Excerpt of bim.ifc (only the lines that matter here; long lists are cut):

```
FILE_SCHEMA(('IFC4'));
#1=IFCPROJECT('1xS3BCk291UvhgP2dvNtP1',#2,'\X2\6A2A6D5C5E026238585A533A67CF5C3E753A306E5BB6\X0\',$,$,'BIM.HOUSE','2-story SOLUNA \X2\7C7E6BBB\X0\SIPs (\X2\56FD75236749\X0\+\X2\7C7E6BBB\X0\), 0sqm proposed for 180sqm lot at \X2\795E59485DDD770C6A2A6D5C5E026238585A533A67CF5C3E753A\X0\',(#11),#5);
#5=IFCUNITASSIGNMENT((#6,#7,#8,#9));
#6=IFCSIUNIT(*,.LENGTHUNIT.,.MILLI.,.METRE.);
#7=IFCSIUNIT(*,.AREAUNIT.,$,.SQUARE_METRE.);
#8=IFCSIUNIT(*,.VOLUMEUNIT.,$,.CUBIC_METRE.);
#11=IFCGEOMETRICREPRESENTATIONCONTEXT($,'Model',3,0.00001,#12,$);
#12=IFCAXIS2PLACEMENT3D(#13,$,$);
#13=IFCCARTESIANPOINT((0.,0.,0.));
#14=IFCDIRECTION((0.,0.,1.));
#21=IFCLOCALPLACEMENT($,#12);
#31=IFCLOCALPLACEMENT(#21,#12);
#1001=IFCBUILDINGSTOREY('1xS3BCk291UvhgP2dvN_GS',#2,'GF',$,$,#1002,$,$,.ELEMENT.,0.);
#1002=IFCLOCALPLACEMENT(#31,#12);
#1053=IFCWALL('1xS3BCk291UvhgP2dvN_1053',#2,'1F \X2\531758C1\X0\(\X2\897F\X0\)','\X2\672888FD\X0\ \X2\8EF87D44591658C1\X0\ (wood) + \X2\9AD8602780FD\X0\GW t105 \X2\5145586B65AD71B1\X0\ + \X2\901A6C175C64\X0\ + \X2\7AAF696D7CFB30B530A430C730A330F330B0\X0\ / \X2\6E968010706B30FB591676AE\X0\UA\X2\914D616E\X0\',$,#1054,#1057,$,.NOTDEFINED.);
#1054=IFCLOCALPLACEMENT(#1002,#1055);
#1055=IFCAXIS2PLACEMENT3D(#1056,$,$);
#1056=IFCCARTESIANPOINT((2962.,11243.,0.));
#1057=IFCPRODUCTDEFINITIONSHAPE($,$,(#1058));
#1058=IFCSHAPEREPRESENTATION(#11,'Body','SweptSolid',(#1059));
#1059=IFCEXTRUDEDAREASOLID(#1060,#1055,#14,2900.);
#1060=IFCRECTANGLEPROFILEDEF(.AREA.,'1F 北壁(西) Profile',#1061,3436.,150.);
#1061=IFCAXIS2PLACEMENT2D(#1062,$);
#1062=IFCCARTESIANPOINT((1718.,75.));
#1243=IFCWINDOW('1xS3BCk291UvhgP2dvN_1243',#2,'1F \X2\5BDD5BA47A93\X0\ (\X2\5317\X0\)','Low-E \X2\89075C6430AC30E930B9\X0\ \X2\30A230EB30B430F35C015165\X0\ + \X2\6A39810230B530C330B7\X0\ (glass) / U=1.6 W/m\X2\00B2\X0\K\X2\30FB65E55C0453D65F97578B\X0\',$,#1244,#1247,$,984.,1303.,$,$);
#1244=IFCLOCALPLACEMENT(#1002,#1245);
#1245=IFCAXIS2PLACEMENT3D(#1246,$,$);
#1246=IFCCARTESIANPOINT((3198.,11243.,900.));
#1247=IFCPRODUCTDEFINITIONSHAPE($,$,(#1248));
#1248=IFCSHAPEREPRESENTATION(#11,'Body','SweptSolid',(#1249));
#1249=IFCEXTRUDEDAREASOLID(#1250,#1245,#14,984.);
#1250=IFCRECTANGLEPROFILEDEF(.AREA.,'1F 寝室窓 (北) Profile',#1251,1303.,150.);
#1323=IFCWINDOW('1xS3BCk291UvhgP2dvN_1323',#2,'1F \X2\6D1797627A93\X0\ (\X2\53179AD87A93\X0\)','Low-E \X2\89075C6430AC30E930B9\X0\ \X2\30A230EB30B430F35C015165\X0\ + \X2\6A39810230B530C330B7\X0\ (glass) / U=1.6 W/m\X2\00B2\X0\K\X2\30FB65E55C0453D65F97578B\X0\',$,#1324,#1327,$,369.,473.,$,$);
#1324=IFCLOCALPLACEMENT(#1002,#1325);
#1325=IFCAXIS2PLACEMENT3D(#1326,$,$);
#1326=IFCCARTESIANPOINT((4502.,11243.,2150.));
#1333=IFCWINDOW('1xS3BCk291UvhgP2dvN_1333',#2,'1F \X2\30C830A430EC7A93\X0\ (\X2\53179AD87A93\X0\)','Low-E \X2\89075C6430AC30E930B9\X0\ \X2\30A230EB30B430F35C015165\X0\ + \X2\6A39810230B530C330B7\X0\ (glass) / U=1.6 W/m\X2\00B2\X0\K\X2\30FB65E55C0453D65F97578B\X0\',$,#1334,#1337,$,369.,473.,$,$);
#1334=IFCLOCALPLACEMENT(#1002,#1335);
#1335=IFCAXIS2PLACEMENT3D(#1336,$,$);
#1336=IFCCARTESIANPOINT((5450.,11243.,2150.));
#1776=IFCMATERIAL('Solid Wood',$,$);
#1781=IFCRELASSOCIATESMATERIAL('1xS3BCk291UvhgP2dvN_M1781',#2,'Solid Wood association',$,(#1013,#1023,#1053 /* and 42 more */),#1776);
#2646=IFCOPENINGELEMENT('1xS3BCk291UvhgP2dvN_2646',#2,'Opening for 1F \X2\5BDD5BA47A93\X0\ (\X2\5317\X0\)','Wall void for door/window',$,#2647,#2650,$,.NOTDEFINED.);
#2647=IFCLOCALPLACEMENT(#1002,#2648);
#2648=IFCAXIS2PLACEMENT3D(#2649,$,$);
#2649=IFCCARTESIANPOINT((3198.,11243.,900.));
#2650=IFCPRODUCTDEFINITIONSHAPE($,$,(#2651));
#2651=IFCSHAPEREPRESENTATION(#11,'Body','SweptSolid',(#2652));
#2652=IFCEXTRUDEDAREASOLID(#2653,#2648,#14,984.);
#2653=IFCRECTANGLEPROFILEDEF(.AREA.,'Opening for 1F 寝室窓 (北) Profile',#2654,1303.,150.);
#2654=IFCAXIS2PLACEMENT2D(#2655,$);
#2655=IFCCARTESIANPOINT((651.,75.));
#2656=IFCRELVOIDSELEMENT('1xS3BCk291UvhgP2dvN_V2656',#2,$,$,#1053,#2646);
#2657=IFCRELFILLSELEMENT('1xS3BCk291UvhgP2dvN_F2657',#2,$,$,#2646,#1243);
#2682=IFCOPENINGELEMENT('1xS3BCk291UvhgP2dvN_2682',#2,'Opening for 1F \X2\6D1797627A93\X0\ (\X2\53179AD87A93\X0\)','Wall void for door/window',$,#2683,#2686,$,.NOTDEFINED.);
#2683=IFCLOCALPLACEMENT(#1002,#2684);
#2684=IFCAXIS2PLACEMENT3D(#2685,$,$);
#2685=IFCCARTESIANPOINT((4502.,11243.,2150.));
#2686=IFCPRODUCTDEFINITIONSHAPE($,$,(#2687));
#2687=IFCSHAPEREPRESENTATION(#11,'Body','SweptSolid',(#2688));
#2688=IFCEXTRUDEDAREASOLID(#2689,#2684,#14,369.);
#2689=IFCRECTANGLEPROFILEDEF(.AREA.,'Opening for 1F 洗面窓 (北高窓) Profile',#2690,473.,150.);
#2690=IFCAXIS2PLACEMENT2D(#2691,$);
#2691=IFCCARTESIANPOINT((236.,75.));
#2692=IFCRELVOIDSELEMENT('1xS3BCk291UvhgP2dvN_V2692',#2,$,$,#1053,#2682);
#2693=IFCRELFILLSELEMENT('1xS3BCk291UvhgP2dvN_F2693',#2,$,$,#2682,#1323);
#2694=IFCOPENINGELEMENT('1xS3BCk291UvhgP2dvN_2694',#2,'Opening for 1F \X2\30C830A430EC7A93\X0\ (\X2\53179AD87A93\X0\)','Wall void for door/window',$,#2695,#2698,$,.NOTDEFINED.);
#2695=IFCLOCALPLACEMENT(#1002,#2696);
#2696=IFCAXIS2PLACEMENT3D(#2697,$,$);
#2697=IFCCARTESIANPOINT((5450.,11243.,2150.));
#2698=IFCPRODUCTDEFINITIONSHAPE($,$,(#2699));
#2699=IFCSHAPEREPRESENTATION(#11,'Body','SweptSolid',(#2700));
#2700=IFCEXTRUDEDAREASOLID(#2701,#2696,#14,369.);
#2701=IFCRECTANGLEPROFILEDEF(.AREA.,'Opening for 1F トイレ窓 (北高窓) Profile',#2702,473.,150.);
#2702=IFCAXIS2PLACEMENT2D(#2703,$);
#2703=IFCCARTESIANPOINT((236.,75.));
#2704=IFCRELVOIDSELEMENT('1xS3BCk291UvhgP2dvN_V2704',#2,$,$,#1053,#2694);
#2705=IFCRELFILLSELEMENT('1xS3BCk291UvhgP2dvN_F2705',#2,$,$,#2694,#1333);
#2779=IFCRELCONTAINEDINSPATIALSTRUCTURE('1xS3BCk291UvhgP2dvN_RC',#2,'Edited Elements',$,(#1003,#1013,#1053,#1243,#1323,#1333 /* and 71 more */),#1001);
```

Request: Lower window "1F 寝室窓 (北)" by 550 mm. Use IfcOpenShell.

```python
import numpy as np
import ifcopenshell
import ifcopenshell.api.geometry
import ifcopenshell.util.placement
import ifcopenshell.util.unit

model = ifcopenshell.open("bim.ifc")
unit_scale = ifcopenshell.util.unit.calculate_unit_scale(model)

window = model.by_guid("1xS3BCk291UvhgP2dvN_1243")
opening = window.FillsVoids[0].RelatingOpeningElement
dz = -0.55 / unit_scale

shift = np.array([0.0, 0.0, dz])
# The window is not placed relative to its opening, so move both.
for product in (opening, window):
    matrix = ifcopenshell.util.placement.get_local_placement(product.ObjectPlacement)
    matrix[:3, 3] += shift
    ifcopenshell.api.geometry.edit_object_placement(model, product=product, matrix=matrix, is_si=False)

print(f"moved by {dz * unit_scale:+.3f} m")

model.write("bim_rev.ifc")
```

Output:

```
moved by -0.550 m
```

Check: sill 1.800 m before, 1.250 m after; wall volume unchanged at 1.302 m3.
